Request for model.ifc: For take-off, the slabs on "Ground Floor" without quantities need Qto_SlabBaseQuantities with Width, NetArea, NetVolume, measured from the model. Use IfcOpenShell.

First a look at what the model holds.

```python
import ifcopenshell
import ifcopenshell.util.element
import ifcopenshell.util.unit

model = ifcopenshell.open("model.ifc")
print(model.schema)
for unit_type in ("LENGTHUNIT", "AREAUNIT", "VOLUMEUNIT"):
    print(unit_type, ifcopenshell.util.unit.calculate_unit_scale(model, unit_type))
storey = next(s for s in model.by_type("IfcBuildingStorey") if s.Name == "Ground Floor")
slabs = [e for e in ifcopenshell.util.element.get_decomposition(storey) if e.is_a("IfcSlab")]
for e in sorted(slabs, key=lambda e: e.id()):
    print(e.id(), e.is_a(), e.Name, list(ifcopenshell.util.element.get_psets(e, qtos_only=True)), sep=" | ")
```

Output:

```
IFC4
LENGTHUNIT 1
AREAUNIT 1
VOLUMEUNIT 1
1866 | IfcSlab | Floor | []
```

```python
import ifcopenshell
import ifcopenshell.api.pset
import ifcopenshell.geom
import ifcopenshell.util.element
import ifcopenshell.util.shape
import ifcopenshell.util.unit

model = ifcopenshell.open("model.ifc")
unit_scale = ifcopenshell.util.unit.calculate_unit_scale(model)
area_scale = ifcopenshell.util.unit.calculate_unit_scale(model, "AREAUNIT")
volume_scale = ifcopenshell.util.unit.calculate_unit_scale(model, "VOLUMEUNIT")
settings = ifcopenshell.geom.settings()

storey = next(s for s in model.by_type("IfcBuildingStorey") if s.Name == "Ground Floor")
slabs = [e for e in ifcopenshell.util.element.get_decomposition(storey) if e.is_a("IfcSlab")]

for e in sorted(slabs, key=lambda e: e.id()):
    if ifcopenshell.util.element.get_psets(e, qtos_only=True, should_inherit=False):
        continue
    # Geometry comes back in metres, in the element's own axes.
    shape = ifcopenshell.geom.create_shape(settings, e)
    values = {
        "Width": ifcopenshell.util.shape.get_z(shape.geometry) / unit_scale,
        "NetArea": ifcopenshell.util.shape.get_footprint_area(shape.geometry) / area_scale,
        "NetVolume": ifcopenshell.util.shape.get_volume(shape.geometry) / volume_scale,
    }
    qto = ifcopenshell.api.pset.add_qto(model, product=e, name="Qto_SlabBaseQuantities")
    ifcopenshell.api.pset.edit_qto(model, qto=qto, properties=values)
    print(e.id(), {k: round(v, 3) for k, v in values.items()})

model.write("model_rev.ifc")
```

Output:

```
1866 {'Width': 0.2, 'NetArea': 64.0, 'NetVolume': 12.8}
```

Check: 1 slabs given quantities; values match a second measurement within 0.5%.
